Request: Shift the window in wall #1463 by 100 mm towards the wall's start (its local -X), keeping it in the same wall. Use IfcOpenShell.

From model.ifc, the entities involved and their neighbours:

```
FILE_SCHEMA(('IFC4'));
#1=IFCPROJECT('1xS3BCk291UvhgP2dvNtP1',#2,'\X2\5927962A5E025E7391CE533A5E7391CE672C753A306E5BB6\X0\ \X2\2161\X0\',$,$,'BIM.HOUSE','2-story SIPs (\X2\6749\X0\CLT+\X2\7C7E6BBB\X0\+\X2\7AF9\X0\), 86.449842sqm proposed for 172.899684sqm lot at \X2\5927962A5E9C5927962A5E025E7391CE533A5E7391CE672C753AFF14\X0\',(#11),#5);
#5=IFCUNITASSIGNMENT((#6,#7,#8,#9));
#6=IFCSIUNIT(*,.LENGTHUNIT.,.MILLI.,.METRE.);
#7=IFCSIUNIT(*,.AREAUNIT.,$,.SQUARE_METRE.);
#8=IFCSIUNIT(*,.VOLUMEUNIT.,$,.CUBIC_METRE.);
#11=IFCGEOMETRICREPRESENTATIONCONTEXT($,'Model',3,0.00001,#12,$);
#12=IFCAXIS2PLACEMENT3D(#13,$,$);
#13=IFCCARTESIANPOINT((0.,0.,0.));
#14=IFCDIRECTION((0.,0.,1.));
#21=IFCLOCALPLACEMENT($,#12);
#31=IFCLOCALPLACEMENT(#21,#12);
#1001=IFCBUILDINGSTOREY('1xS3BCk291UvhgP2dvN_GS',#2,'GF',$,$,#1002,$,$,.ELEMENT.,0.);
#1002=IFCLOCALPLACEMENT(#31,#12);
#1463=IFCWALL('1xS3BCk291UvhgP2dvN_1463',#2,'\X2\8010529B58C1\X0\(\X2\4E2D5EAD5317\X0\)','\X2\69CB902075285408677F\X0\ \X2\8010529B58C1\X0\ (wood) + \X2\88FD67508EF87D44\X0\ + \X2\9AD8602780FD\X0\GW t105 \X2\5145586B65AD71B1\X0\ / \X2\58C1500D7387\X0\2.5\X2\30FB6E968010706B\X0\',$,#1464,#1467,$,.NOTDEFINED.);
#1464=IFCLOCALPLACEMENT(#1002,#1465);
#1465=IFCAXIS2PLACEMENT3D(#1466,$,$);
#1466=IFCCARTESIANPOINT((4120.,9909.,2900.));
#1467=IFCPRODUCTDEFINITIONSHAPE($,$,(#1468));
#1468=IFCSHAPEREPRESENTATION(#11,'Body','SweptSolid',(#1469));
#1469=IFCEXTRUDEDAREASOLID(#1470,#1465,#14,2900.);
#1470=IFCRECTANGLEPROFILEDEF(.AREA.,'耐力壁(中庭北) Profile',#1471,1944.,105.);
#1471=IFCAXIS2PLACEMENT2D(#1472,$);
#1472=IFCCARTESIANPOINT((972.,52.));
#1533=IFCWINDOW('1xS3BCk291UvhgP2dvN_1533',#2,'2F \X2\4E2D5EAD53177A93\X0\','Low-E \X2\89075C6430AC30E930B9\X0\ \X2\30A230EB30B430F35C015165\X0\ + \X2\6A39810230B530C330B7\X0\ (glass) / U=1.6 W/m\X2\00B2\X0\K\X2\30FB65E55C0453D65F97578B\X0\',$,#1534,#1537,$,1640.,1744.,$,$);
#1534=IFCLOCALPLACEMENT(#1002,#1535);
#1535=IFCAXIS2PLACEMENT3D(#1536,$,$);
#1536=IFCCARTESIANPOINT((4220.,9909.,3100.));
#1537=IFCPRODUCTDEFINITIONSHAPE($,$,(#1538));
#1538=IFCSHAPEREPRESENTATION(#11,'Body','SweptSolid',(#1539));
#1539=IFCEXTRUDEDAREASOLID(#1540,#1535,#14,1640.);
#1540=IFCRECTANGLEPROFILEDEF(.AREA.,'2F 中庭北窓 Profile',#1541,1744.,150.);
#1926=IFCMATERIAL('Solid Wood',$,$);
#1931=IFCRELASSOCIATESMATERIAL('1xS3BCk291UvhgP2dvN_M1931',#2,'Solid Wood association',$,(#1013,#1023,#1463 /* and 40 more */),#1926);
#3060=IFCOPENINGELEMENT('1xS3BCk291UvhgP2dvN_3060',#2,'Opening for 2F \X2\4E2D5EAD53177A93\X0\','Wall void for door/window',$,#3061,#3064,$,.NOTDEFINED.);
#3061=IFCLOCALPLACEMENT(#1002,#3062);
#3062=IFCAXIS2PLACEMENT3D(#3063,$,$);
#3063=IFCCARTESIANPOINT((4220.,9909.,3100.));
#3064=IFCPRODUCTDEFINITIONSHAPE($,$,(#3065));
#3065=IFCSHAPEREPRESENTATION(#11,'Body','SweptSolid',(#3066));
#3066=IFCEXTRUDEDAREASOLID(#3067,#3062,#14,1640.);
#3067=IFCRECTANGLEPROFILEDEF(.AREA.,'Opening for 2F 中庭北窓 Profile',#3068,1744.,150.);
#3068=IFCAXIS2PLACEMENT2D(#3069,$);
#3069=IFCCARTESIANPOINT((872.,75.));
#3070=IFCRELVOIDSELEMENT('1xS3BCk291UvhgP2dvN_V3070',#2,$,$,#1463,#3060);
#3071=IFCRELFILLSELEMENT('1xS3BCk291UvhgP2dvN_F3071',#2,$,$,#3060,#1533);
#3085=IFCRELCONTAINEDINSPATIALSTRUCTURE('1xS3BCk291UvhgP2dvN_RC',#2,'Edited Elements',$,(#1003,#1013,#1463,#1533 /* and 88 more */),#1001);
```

```python
import ifcopenshell
import ifcopenshell.api.geometry
import ifcopenshell.util.placement
import ifcopenshell.util.unit

model = ifcopenshell.open("model.ifc")
unit_scale = ifcopenshell.util.unit.calculate_unit_scale(model)

window = model.by_id(1533)
opening = window.FillsVoids[0].RelatingOpeningElement
wall = opening.VoidsElements[0].RelatingBuildingElement

wall_matrix = ifcopenshell.util.placement.get_local_placement(wall.ObjectPlacement)
shift = wall_matrix[:3, 0] * -0.1 / unit_scale
before = ifcopenshell.util.placement.get_local_placement(window.ObjectPlacement)[:3, 3].copy()

# The window is not placed relative to its opening, so move both.
for product in (opening, window):
    matrix = ifcopenshell.util.placement.get_local_placement(product.ObjectPlacement)
    matrix[:3, 3] += shift
    ifcopenshell.api.geometry.edit_object_placement(model, product=product, matrix=matrix, is_si=False)

after = ifcopenshell.util.placement.get_local_placement(window.ObjectPlacement)[:3, 3]
print("window moved by", (after - before).round(3) + 0.0)

model.write("model_v2.ifc")
```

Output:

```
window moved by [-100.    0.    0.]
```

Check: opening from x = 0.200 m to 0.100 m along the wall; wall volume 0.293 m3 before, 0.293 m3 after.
